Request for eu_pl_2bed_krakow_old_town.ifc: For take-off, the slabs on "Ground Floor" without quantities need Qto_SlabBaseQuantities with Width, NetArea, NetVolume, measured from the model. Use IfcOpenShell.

First a look at what the model holds.

```python
import ifcopenshell
import ifcopenshell.util.element
import ifcopenshell.util.unit

model = ifcopenshell.open("eu_pl_2bed_krakow_old_town.ifc")
print(model.schema)
for unit_type in ("LENGTHUNIT", "AREAUNIT", "VOLUMEUNIT"):
    print(unit_type, ifcopenshell.util.unit.calculate_unit_scale(model, unit_type))
storey = next(s for s in model.by_type("IfcBuildingStorey") if s.Name == "Ground Floor")
slabs = [e for e in ifcopenshell.util.element.get_decomposition(storey) if e.is_a("IfcSlab")]
for e in sorted(slabs, key=lambda e: e.id()):
    print(e.id(), e.is_a(), e.Name, list(ifcopenshell.util.element.get_psets(e, qtos_only=True)), sep=" | ")
```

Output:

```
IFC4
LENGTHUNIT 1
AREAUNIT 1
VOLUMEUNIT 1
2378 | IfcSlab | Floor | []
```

```python
import ifcopenshell
import ifcopenshell.api.pset
import ifcopenshell.geom
import ifcopenshell.util.element
import ifcopenshell.util.shape
import ifcopenshell.util.unit

model = ifcopenshell.open("eu_pl_2bed_krakow_old_town.ifc")
unit_scale = ifcopenshell.util.unit.calculate_unit_scale(model)
area_scale = ifcopenshell.util.unit.calculate_unit_scale(model, "AREAUNIT")
volume_scale = ifcopenshell.util.unit.calculate_unit_scale(model, "VOLUMEUNIT")
settings = ifcopenshell.geom.settings()

storey = next(s for s in model.by_type("IfcBuildingStorey") if s.Name == "Ground Floor")
slabs = [e for e in ifcopenshell.util.element.get_decomposition(storey) if e.is_a("IfcSlab")]

for e in sorted(slabs, key=lambda e: e.id()):
    if ifcopenshell.util.element.get_psets(e, qtos_only=True, should_inherit=False):
        continue
    # Geometry comes back in metres, in the element's own axes.
    shape = ifcopenshell.geom.create_shape(settings, e)
    values = {
        "Width": ifcopenshell.util.shape.get_z(shape.geometry) / unit_scale,
        "NetArea": ifcopenshell.util.shape.get_footprint_area(shape.geometry) / area_scale,
        "NetVolume": ifcopenshell.util.shape.get_volume(shape.geometry) / volume_scale,
    }
    qto = ifcopenshell.api.pset.add_qto(model, product=e, name="Qto_SlabBaseQuantities")
    ifcopenshell.api.pset.edit_qto(model, qto=qto, properties=values)
    print(e.id(), {k: round(v, 3) for k, v in values.items()})

model.write("eu_pl_2bed_krakow_old_town_rev.ifc")
```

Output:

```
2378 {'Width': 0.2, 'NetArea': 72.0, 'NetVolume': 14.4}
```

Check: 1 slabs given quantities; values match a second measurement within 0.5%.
